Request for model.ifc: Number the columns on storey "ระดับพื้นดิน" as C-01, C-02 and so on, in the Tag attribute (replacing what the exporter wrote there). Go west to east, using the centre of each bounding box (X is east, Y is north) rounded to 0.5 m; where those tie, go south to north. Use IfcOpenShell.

First a look at what the model holds.

```python
import ifcopenshell
import ifcopenshell.util.element
import ifcopenshell.util.placement

model = ifcopenshell.open("model.ifc")
print(model.schema)
storey = next(s for s in model.by_type("IfcBuildingStorey") if s.Name == "ระดับพื้นดิน")
columns = [e for e in ifcopenshell.util.element.get_decomposition(storey) if e.is_a("IfcColumn")]
for e in sorted(columns, key=lambda e: e.id()):
    origin = ifcopenshell.util.placement.get_local_placement(e.ObjectPlacement)[:3, 3]
    print(e.id(), e.Tag, e.Name, origin.round(2) + 0.0, sep=" | ")
```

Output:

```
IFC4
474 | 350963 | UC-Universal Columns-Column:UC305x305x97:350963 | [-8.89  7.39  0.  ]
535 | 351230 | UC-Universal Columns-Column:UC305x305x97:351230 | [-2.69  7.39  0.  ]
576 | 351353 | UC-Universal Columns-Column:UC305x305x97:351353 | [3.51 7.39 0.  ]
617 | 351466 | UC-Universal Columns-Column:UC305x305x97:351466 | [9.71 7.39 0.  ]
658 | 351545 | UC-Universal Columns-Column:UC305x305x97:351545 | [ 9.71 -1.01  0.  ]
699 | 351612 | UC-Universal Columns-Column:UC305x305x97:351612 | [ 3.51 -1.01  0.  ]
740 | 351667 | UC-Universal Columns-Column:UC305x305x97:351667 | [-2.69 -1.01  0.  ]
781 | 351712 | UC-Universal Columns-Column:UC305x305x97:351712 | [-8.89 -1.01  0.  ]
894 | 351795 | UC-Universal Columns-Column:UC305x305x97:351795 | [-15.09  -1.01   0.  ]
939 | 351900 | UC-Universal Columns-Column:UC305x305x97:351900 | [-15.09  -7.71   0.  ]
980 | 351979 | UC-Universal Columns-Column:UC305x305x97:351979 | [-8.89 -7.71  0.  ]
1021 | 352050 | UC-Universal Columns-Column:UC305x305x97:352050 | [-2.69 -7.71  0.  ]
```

```python
import ifcopenshell
import ifcopenshell.geom
import ifcopenshell.util.element
import ifcopenshell.util.shape

model = ifcopenshell.open("model.ifc")
settings = ifcopenshell.geom.settings()
settings.set("use-world-coords", True)


def centre(element):
    shape = ifcopenshell.geom.create_shape(settings, element)
    return ifcopenshell.util.shape.get_bbox_centroid(shape.geometry)


storey = next(s for s in model.by_type("IfcBuildingStorey") if s.Name == "ระดับพื้นดิน")
columns = [e for e in ifcopenshell.util.element.get_decomposition(storey) if e.is_a("IfcColumn")]

# Insertion points can sit at a corner or the storey origin, so sort by the geometry (in metres).
centres = {e: centre(e) for e in columns}
columns.sort(key=lambda e: (round(centres[e][0] / 0.5), centres[e][1]))

for i, e in enumerate(columns, start=1):
    number = f"C-{i:02d}"
    e.Tag = number
    print(e.id(), number)

model.write("model-out.ifc")
```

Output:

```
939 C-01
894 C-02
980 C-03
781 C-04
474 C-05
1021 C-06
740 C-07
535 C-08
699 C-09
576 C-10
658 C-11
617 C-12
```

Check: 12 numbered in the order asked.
